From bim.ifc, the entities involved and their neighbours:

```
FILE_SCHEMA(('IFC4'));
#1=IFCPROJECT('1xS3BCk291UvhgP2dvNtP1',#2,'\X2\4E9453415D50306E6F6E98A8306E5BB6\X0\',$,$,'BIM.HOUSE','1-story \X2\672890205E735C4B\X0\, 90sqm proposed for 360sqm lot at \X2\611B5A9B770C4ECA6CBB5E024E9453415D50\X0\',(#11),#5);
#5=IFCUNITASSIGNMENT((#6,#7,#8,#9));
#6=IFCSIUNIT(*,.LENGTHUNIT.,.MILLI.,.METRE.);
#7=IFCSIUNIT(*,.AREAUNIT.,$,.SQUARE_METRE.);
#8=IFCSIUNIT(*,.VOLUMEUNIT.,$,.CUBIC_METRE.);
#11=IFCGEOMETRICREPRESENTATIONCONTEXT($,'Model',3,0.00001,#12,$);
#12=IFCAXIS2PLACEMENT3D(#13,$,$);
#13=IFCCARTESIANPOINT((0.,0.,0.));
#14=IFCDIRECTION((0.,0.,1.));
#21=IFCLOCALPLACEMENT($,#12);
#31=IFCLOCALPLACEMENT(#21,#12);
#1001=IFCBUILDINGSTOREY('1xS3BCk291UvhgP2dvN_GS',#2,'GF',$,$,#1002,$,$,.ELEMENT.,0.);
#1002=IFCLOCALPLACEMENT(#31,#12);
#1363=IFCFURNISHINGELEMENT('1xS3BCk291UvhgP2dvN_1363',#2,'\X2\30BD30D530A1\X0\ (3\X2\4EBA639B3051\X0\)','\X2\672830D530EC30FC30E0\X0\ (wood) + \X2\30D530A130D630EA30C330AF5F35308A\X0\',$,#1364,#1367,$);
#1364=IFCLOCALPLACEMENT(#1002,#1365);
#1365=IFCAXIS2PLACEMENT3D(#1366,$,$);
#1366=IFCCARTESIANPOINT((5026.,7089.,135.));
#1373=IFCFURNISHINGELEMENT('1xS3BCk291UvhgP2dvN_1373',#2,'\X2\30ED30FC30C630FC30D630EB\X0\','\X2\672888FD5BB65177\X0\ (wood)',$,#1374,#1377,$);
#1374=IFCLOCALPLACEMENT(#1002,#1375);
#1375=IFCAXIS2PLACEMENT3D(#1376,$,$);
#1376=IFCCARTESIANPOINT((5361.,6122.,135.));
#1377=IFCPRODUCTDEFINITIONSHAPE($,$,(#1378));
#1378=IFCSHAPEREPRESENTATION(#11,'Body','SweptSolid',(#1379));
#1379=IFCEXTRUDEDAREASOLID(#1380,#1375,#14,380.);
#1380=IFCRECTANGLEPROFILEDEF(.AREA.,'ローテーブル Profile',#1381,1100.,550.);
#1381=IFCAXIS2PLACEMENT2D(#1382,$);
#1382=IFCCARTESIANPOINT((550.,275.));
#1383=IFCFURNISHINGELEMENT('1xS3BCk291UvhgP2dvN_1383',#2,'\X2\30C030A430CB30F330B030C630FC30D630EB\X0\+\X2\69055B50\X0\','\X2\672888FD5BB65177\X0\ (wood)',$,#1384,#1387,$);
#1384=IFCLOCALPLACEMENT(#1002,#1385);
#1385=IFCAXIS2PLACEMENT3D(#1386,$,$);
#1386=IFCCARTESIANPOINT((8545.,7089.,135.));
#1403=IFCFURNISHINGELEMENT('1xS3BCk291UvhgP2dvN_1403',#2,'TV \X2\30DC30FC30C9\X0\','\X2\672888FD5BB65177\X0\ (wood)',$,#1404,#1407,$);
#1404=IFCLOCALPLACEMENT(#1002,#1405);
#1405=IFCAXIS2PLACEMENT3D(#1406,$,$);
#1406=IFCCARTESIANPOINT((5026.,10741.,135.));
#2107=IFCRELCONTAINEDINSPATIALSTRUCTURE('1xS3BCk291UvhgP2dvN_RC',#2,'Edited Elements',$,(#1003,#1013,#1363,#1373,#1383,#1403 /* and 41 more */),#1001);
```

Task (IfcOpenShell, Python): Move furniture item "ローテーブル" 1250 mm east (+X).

```python
import ifcopenshell
import ifcopenshell.api.geometry
import ifcopenshell.util.placement
import ifcopenshell.util.unit

model = ifcopenshell.open("bim.ifc")
unit_scale = ifcopenshell.util.unit.calculate_unit_scale(model)

item = model.by_id(1373)
matrix = ifcopenshell.util.placement.get_local_placement(item.ObjectPlacement)
matrix[0, 3] += 1.25 / unit_scale
ifcopenshell.api.geometry.edit_object_placement(model, product=item, matrix=matrix, is_si=False)

print(ifcopenshell.util.placement.get_local_placement(item.ObjectPlacement).round(3) + 0.0)

model.write("bim-out.ifc")
```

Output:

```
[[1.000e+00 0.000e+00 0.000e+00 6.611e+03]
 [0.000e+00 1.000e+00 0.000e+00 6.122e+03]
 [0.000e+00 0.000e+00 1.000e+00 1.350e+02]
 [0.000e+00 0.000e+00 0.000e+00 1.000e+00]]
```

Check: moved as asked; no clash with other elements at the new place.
